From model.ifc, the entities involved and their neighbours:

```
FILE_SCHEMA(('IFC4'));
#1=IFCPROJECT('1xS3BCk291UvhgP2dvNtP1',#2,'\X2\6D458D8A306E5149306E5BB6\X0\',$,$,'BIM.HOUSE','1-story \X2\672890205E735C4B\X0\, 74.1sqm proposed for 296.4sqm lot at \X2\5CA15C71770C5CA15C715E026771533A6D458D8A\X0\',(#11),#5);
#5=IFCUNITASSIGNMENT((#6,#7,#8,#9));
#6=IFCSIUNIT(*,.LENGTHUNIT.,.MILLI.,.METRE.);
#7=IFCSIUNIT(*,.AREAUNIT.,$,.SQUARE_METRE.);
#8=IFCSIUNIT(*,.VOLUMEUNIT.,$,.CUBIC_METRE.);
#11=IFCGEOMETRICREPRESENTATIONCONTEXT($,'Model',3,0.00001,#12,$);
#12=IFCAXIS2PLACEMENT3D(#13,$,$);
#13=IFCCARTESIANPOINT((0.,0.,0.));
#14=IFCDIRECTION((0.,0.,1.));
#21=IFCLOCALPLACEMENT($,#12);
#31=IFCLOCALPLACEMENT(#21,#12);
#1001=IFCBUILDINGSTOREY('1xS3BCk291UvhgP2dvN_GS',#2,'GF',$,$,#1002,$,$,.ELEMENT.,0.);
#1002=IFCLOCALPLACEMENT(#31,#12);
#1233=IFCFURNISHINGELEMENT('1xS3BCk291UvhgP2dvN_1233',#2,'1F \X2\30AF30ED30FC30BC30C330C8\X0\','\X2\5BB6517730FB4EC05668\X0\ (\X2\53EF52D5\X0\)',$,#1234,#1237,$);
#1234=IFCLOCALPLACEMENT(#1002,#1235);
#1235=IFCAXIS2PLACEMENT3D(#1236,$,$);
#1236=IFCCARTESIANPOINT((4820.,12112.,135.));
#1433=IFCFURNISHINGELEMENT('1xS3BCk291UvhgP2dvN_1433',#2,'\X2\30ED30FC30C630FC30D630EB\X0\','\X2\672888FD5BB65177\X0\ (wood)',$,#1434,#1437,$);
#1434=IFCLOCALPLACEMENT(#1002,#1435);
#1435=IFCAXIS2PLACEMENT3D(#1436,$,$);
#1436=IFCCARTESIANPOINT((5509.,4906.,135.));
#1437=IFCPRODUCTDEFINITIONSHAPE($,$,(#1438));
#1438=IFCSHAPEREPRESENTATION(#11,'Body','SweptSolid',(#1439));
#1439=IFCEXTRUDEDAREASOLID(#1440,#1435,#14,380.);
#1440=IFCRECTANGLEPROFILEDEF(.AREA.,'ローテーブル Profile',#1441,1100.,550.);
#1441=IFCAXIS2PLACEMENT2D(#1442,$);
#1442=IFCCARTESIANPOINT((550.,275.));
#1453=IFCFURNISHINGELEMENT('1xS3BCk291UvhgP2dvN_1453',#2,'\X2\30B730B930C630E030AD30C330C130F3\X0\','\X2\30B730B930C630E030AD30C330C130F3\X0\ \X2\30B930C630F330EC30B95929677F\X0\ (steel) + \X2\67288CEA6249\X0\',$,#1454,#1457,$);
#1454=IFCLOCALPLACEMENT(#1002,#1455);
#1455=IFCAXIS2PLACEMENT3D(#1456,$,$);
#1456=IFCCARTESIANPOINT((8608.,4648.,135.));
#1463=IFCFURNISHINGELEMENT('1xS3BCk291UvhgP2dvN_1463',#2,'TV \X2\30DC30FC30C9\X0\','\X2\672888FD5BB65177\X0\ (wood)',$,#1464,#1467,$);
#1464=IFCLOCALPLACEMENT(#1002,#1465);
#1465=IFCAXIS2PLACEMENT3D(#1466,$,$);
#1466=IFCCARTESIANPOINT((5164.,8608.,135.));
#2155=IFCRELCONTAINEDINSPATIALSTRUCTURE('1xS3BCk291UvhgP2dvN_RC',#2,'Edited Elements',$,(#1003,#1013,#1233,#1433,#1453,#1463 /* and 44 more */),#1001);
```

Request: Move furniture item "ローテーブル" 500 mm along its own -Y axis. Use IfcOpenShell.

```python
import ifcopenshell
import ifcopenshell.api.geometry
import ifcopenshell.util.placement

model = ifcopenshell.open("model.ifc")

item = model.by_guid("1xS3BCk291UvhgP2dvN_1433")
matrix = ifcopenshell.util.placement.get_local_placement(item.ObjectPlacement)
matrix[:3, 3] -= matrix[:3, 1] * 500.0
ifcopenshell.api.geometry.edit_object_placement(model, product=item, matrix=matrix, is_si=False)

print(ifcopenshell.util.placement.get_local_placement(item.ObjectPlacement).round(3) + 0.0)

model.write("model_rev.ifc")
```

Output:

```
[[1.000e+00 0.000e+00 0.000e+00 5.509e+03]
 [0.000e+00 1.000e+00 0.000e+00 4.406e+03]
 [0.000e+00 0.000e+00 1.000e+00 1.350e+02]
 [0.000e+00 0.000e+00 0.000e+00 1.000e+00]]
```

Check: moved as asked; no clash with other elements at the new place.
